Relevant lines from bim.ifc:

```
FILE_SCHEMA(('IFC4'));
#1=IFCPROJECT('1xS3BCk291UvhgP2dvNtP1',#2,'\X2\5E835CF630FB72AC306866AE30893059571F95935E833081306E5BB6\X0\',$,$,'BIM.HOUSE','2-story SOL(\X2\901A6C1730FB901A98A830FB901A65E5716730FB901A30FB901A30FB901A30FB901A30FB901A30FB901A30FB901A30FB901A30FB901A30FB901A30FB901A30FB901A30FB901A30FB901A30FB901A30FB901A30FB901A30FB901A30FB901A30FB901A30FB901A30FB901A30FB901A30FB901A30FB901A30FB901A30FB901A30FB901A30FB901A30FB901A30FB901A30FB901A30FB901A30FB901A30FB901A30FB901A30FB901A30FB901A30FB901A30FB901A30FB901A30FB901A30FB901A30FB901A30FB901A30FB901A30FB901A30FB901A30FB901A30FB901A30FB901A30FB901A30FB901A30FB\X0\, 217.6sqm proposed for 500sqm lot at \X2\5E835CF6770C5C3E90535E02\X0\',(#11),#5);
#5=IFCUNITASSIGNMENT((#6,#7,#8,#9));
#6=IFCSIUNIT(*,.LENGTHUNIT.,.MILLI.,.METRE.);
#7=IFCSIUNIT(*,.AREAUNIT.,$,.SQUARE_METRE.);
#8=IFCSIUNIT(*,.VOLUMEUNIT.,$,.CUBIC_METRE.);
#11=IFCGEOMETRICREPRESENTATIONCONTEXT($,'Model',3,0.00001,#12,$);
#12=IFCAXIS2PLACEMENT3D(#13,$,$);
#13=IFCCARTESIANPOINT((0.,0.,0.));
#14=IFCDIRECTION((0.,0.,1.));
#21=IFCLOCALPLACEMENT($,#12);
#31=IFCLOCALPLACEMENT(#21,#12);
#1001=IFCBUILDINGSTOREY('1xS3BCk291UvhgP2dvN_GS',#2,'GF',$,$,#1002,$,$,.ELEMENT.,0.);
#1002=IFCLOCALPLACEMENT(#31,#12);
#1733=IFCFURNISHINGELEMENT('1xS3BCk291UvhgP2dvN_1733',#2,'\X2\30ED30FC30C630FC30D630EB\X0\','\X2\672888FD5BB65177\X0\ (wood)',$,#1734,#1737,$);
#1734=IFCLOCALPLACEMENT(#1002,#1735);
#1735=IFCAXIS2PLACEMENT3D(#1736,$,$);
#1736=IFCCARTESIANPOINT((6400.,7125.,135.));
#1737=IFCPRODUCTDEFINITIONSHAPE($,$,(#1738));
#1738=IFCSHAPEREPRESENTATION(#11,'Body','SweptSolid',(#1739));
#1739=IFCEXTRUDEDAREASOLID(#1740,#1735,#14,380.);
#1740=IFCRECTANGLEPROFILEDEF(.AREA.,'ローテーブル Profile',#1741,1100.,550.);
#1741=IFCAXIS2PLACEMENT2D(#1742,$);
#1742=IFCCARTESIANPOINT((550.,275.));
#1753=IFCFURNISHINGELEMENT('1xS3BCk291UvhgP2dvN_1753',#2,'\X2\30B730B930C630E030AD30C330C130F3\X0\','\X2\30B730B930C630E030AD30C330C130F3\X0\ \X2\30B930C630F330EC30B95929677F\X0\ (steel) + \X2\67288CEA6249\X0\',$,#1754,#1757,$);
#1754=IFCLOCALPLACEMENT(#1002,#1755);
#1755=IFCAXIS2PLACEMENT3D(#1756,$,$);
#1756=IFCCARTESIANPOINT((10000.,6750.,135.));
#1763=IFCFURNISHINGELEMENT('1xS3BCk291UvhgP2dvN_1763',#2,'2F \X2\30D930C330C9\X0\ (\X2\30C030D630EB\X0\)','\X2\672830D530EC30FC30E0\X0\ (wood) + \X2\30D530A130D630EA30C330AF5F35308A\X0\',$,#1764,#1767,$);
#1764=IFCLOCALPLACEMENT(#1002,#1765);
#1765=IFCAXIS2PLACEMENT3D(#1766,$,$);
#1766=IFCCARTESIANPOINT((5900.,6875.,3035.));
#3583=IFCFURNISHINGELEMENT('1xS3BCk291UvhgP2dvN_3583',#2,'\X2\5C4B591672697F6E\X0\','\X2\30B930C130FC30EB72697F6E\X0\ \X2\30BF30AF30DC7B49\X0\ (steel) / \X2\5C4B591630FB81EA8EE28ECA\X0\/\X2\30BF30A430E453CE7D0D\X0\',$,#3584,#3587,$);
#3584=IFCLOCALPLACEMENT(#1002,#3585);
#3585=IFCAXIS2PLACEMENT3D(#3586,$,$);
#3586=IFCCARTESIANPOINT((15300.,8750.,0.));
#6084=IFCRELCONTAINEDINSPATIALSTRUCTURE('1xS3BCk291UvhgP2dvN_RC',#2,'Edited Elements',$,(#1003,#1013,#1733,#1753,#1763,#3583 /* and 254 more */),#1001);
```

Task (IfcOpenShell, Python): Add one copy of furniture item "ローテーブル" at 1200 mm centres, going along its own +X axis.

```python
import ifcopenshell
import ifcopenshell.api.geometry
import ifcopenshell.api.root
import ifcopenshell.util.element
import ifcopenshell.util.placement
import ifcopenshell.util.unit

model = ifcopenshell.open("bim.ifc")
unit_scale = ifcopenshell.util.unit.calculate_unit_scale(model)


def reuse_history(source, copy):
    """copy_class also copies each property set's owner history, people and application; keep the originals."""
    for rel in copy.IsDefinedBy:
        if rel.is_a("IfcRelDefinesByProperties") and (history := rel.RelatingPropertyDefinition.OwnerHistory):
            rel.RelatingPropertyDefinition.OwnerHistory = source.OwnerHistory
            ifcopenshell.util.element.remove_deep2(model, history)


source = model.by_id(1733)
base = ifcopenshell.util.placement.get_local_placement(source.ObjectPlacement)
step = base[:3, 0] * 1.2 / unit_scale

for i in range(1, 2):
    copy = ifcopenshell.api.root.copy_class(model, product=source)
    copy.Representation = ifcopenshell.util.element.copy_deep(
        model, source.Representation, exclude=["IfcGeometricRepresentationContext", "IfcRepresentationMap"]
    )
    reuse_history(source, copy)
    matrix = base.copy()
    matrix[:3, 3] += i * step
    print("added at", matrix[:3, 3].round(3) + 0.0)
    ifcopenshell.api.geometry.edit_object_placement(model, product=copy, matrix=matrix, is_si=False)

model.write("bim_edited.ifc")
```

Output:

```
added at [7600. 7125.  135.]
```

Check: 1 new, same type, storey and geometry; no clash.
